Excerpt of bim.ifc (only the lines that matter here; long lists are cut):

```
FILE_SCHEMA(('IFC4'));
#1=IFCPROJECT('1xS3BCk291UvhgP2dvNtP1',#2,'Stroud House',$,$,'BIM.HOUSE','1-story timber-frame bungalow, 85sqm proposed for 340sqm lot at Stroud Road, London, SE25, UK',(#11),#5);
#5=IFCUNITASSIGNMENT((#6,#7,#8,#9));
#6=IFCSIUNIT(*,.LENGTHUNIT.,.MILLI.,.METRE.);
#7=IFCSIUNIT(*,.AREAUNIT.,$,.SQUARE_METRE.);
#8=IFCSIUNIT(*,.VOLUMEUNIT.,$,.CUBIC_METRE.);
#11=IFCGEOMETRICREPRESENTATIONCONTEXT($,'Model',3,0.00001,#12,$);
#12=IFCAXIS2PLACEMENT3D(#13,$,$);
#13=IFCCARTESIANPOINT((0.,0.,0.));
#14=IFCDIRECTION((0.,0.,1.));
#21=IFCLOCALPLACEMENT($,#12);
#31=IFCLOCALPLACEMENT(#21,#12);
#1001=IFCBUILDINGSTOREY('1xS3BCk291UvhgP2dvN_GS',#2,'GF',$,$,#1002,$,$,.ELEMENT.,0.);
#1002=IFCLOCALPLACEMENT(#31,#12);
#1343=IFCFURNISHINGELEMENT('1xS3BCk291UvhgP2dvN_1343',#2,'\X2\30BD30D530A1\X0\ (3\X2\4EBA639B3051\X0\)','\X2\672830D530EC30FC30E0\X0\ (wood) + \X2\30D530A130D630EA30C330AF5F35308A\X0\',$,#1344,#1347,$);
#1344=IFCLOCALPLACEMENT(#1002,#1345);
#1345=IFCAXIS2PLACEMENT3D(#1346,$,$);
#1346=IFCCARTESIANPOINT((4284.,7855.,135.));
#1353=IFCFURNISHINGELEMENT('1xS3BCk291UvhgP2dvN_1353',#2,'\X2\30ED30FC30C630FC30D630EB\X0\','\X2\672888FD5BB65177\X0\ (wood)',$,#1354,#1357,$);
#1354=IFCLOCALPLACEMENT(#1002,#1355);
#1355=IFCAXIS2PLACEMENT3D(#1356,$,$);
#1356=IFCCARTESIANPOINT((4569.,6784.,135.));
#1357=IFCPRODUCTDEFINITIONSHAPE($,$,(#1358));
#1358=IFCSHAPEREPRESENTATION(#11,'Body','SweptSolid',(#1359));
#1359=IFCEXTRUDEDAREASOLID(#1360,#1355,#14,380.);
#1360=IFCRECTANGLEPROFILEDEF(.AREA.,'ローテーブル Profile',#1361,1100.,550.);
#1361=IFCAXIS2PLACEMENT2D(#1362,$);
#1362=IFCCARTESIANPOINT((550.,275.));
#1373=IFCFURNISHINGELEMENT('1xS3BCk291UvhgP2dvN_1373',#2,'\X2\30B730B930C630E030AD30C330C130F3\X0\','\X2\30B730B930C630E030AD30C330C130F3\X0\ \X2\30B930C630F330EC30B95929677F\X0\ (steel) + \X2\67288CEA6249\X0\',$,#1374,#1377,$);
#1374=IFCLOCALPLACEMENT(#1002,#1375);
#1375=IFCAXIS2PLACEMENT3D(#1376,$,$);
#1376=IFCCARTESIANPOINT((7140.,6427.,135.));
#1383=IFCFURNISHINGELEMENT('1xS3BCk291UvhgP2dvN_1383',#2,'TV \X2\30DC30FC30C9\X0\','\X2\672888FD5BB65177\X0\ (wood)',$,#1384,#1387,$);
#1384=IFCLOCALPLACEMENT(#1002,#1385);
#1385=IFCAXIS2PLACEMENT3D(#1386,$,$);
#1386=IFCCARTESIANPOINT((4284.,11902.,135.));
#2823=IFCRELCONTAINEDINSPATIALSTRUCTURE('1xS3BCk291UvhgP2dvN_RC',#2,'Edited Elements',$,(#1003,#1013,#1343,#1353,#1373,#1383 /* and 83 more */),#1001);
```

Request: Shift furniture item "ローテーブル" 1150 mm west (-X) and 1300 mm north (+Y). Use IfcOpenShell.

```python
import ifcopenshell
import ifcopenshell.api.geometry
import ifcopenshell.util.placement

model = ifcopenshell.open("bim.ifc")

item = model.by_guid("1xS3BCk291UvhgP2dvN_1353")
matrix = ifcopenshell.util.placement.get_local_placement(item.ObjectPlacement)
matrix[0, 3] -= 1150.0
matrix[1, 3] += 1300.0
ifcopenshell.api.geometry.edit_object_placement(model, product=item, matrix=matrix, is_si=False)

print(ifcopenshell.util.placement.get_local_placement(item.ObjectPlacement).round(3) + 0.0)

model.write("bim_updated.ifc")
```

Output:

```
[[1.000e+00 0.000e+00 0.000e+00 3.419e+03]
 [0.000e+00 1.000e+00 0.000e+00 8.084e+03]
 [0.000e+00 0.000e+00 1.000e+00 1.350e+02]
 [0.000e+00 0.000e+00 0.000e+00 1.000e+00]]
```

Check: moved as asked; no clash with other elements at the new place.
